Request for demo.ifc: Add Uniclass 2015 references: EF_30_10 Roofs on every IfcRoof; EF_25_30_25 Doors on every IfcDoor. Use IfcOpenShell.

First a look at what the model holds.

```python
import ifcopenshell

model = ifcopenshell.open("demo.ifc")
print(model.schema)
print("classifications:", [c.Name for c in model.by_type("IfcClassification")])
for ifc_class in ("IfcDoor", "IfcRoof", "IfcStair", "IfcWall", "IfcWindow"):
    print(ifc_class, len(model.by_type(ifc_class)))
```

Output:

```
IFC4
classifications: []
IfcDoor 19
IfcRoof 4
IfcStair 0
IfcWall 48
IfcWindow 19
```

```python
import ifcopenshell
import ifcopenshell.api.classification

model = ifcopenshell.open("demo.ifc")

system = ifcopenshell.api.classification.add_classification(model, classification="Uniclass 2015")

codes = {
    "IfcRoof": ("EF_30_10", "Roofs"),
    "IfcDoor": ("EF_25_30_25", "Doors"),
}
for ifc_class, (code, name) in codes.items():
    products = model.by_type(ifc_class)
    ifcopenshell.api.classification.add_reference(
        model, products=products, classification=system, identification=code, name=name
    )
    print(code, len(products))

model.write("demo_updated.ifc")
```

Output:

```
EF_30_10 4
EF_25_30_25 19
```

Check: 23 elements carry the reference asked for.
